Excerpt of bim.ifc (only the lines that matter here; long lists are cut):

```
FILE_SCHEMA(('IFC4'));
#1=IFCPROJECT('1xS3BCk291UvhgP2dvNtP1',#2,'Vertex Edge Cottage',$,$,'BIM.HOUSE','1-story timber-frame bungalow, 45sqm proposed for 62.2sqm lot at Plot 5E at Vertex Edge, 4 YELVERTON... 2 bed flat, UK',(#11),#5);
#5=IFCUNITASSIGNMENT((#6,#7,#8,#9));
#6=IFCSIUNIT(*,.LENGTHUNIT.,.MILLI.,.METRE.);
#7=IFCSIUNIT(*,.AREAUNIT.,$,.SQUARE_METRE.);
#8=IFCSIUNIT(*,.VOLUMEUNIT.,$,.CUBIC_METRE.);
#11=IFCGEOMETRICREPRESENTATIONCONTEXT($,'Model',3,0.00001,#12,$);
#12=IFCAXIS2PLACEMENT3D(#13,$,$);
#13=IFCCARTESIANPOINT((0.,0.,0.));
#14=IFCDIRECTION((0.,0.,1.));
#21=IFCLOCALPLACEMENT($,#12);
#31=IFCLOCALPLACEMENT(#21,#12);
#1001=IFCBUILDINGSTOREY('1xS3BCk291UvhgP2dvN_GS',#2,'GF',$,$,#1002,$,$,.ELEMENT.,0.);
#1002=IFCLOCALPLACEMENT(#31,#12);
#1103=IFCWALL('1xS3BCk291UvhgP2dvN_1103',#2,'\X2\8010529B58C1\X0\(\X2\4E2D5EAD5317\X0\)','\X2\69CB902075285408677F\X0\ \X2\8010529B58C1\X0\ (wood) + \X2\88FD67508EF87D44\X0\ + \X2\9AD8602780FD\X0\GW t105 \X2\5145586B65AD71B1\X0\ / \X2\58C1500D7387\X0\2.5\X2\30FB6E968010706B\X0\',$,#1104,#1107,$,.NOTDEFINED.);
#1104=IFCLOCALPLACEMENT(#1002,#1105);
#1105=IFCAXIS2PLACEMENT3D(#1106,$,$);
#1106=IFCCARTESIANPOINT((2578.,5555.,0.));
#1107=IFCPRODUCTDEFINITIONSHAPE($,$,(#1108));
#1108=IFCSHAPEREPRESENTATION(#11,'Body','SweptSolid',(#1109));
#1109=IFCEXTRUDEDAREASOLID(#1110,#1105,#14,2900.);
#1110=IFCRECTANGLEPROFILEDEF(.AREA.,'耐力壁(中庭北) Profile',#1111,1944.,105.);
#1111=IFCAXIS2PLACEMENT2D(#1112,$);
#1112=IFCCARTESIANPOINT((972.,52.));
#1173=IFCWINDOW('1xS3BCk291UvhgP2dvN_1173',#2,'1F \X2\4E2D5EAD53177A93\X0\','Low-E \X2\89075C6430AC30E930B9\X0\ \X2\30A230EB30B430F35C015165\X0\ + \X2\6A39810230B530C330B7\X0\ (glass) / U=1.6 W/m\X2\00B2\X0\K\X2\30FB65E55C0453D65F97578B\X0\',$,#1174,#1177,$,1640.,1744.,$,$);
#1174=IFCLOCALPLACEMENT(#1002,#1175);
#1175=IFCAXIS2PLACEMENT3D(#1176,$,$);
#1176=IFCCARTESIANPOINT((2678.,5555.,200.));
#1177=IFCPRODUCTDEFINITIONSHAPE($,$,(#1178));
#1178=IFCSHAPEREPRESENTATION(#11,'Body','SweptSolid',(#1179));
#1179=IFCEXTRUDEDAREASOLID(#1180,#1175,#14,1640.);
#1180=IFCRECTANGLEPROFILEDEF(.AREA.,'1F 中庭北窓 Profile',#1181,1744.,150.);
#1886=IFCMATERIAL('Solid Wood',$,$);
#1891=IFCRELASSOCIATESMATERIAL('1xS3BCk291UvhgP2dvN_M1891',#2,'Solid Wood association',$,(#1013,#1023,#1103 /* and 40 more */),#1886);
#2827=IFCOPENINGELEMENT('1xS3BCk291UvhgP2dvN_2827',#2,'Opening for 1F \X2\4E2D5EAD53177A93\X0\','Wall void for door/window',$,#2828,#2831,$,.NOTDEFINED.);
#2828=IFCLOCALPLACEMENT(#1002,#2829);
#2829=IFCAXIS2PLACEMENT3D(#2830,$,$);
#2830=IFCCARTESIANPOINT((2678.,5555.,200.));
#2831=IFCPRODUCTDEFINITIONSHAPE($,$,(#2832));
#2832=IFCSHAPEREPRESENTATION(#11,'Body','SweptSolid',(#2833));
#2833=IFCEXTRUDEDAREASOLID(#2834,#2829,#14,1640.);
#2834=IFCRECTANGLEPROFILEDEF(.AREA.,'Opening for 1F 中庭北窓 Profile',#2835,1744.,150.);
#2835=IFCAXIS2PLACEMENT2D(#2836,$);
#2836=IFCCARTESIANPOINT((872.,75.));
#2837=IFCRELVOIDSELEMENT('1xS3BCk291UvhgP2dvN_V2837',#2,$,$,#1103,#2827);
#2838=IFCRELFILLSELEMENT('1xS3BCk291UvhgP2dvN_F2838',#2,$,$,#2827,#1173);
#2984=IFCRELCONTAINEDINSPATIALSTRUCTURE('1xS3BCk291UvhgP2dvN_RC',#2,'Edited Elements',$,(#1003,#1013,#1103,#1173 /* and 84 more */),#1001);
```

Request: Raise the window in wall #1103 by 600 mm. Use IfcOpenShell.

```python
import numpy as np
import ifcopenshell
import ifcopenshell.api.geometry
import ifcopenshell.util.placement
import ifcopenshell.util.unit

model = ifcopenshell.open("bim.ifc")
unit_scale = ifcopenshell.util.unit.calculate_unit_scale(model)

window = model.by_guid("1xS3BCk291UvhgP2dvN_1173")
opening = window.FillsVoids[0].RelatingOpeningElement
dz = 0.6 / unit_scale

shift = np.array([0.0, 0.0, dz])
# The window is not placed relative to its opening, so move both.
for product in (opening, window):
    matrix = ifcopenshell.util.placement.get_local_placement(product.ObjectPlacement)
    matrix[:3, 3] += shift
    ifcopenshell.api.geometry.edit_object_placement(model, product=product, matrix=matrix, is_si=False)

print(f"moved by {dz * unit_scale:+.3f} m")

model.write("bim-out.ifc")
```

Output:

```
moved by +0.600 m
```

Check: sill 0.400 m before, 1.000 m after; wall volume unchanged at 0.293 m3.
